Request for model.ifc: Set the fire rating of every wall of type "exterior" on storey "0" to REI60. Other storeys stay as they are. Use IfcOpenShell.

First a look at what the model holds.

```python
import ifcopenshell
import ifcopenshell.util.element

model = ifcopenshell.open("model.ifc")
print(model.schema)
storey = next(s for s in model.by_type("IfcBuildingStorey") if s.Name == "0")
walls = [e for e in ifcopenshell.util.element.get_decomposition(storey) if e.is_a("IfcWall")]
seen = {}
for e in walls:
    element_type = ifcopenshell.util.element.get_type(e)
    key = (element_type.Name if element_type != e and element_type else None, ifcopenshell.util.element.get_pset(e, "Pset_WallCommon", "FireRating"))
    seen[key] = seen.get(key, 0) + 1
for (name, value), count in sorted(seen.items(), key=str):
    print(count, "x", name, "|", value)
```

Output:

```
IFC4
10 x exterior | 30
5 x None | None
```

```python
import ifcopenshell
import ifcopenshell.api.pset
import ifcopenshell.util.element

model = ifcopenshell.open("model.ifc")

storey = next(s for s in model.by_type("IfcBuildingStorey") if s.Name == "0")
walls = [e for e in ifcopenshell.util.element.get_decomposition(storey) if e.is_a("IfcWall")]

count = 0
for e in walls:
    element_type = ifcopenshell.util.element.get_type(e)
    if element_type in (None, e) or element_type.Name != "exterior":
        continue
    # add_pset returns the element's existing set when there is one.
    pset = ifcopenshell.api.pset.add_pset(model, product=e, name="Pset_WallCommon")
    ifcopenshell.api.pset.edit_pset(model, pset=pset, properties={"FireRating": "REI60"})
    count += 1

print(count, "walls updated")

model.write("model-out.ifc")
```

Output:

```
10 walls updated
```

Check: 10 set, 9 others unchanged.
